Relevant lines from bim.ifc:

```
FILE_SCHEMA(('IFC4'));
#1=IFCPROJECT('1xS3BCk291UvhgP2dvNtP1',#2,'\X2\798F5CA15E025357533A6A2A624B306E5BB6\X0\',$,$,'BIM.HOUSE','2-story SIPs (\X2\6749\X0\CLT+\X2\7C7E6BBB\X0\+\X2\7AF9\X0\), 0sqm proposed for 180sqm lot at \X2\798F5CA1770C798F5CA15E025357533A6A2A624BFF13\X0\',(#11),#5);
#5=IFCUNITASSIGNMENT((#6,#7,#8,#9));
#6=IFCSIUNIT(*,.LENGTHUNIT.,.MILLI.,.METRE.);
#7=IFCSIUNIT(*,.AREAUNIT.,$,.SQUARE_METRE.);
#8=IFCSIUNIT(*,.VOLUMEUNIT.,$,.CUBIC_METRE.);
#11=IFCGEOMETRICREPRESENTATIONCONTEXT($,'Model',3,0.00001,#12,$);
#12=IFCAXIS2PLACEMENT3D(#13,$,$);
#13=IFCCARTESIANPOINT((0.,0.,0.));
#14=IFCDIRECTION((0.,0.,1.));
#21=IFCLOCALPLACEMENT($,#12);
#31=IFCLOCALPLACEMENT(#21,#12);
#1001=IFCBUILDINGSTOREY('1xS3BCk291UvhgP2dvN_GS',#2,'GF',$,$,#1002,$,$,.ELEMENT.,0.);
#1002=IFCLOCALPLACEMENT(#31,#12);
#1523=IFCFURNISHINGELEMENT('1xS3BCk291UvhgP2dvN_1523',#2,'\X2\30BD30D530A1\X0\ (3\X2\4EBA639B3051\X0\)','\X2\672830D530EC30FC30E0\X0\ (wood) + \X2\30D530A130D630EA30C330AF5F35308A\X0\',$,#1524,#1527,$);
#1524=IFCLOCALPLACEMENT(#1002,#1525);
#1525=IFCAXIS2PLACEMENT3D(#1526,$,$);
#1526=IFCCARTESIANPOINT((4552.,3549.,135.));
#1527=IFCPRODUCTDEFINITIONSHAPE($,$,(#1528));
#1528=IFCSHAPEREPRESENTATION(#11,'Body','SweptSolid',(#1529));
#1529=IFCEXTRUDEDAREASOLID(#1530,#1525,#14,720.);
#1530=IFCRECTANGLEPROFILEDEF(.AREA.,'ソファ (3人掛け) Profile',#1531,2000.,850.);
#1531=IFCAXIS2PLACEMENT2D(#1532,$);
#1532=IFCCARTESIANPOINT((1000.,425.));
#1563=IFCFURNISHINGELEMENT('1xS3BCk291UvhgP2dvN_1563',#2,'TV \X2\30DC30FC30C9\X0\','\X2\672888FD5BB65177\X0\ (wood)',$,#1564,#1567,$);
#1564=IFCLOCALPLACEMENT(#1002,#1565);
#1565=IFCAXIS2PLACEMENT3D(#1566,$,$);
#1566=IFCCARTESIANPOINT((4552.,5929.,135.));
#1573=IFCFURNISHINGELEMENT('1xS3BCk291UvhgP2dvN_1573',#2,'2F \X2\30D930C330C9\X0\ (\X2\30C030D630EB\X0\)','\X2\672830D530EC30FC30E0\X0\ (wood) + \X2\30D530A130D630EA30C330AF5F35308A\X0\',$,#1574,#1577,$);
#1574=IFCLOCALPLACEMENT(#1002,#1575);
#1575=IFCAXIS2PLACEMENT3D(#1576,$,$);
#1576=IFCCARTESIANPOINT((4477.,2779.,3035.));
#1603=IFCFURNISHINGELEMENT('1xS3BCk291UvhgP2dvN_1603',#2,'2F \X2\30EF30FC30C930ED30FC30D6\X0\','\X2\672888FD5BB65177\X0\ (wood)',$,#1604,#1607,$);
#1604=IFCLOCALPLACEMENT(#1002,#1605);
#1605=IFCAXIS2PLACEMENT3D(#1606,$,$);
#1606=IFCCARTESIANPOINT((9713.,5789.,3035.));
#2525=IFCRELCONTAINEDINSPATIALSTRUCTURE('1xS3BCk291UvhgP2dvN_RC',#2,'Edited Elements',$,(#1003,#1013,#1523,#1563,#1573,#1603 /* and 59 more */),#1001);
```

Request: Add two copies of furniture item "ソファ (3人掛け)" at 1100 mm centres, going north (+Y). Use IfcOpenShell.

```python
import numpy as np
import ifcopenshell
import ifcopenshell.api.geometry
import ifcopenshell.api.root
import ifcopenshell.util.element
import ifcopenshell.util.placement
import ifcopenshell.util.unit

model = ifcopenshell.open("bim.ifc")
unit_scale = ifcopenshell.util.unit.calculate_unit_scale(model)


def reuse_history(source, copy):
    """copy_class also copies each property set's owner history, people and application; keep the originals."""
    for rel in copy.IsDefinedBy:
        if rel.is_a("IfcRelDefinesByProperties") and (history := rel.RelatingPropertyDefinition.OwnerHistory):
            rel.RelatingPropertyDefinition.OwnerHistory = source.OwnerHistory
            ifcopenshell.util.element.remove_deep2(model, history)


source = model.by_guid("1xS3BCk291UvhgP2dvN_1523")
base = ifcopenshell.util.placement.get_local_placement(source.ObjectPlacement)
step = np.array([0.0, 1.0, 0.0]) * 1.1 / unit_scale

for i in range(1, 3):
    copy = ifcopenshell.api.root.copy_class(model, product=source)
    copy.Representation = ifcopenshell.util.element.copy_deep(
        model, source.Representation, exclude=["IfcGeometricRepresentationContext", "IfcRepresentationMap"]
    )
    reuse_history(source, copy)
    matrix = base.copy()
    matrix[:3, 3] += i * step
    print("added at", matrix[:3, 3].round(3) + 0.0)
    ifcopenshell.api.geometry.edit_object_placement(model, product=copy, matrix=matrix, is_si=False)

model.write("bim_edited.ifc")
```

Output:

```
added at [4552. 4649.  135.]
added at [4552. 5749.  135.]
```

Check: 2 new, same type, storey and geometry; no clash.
